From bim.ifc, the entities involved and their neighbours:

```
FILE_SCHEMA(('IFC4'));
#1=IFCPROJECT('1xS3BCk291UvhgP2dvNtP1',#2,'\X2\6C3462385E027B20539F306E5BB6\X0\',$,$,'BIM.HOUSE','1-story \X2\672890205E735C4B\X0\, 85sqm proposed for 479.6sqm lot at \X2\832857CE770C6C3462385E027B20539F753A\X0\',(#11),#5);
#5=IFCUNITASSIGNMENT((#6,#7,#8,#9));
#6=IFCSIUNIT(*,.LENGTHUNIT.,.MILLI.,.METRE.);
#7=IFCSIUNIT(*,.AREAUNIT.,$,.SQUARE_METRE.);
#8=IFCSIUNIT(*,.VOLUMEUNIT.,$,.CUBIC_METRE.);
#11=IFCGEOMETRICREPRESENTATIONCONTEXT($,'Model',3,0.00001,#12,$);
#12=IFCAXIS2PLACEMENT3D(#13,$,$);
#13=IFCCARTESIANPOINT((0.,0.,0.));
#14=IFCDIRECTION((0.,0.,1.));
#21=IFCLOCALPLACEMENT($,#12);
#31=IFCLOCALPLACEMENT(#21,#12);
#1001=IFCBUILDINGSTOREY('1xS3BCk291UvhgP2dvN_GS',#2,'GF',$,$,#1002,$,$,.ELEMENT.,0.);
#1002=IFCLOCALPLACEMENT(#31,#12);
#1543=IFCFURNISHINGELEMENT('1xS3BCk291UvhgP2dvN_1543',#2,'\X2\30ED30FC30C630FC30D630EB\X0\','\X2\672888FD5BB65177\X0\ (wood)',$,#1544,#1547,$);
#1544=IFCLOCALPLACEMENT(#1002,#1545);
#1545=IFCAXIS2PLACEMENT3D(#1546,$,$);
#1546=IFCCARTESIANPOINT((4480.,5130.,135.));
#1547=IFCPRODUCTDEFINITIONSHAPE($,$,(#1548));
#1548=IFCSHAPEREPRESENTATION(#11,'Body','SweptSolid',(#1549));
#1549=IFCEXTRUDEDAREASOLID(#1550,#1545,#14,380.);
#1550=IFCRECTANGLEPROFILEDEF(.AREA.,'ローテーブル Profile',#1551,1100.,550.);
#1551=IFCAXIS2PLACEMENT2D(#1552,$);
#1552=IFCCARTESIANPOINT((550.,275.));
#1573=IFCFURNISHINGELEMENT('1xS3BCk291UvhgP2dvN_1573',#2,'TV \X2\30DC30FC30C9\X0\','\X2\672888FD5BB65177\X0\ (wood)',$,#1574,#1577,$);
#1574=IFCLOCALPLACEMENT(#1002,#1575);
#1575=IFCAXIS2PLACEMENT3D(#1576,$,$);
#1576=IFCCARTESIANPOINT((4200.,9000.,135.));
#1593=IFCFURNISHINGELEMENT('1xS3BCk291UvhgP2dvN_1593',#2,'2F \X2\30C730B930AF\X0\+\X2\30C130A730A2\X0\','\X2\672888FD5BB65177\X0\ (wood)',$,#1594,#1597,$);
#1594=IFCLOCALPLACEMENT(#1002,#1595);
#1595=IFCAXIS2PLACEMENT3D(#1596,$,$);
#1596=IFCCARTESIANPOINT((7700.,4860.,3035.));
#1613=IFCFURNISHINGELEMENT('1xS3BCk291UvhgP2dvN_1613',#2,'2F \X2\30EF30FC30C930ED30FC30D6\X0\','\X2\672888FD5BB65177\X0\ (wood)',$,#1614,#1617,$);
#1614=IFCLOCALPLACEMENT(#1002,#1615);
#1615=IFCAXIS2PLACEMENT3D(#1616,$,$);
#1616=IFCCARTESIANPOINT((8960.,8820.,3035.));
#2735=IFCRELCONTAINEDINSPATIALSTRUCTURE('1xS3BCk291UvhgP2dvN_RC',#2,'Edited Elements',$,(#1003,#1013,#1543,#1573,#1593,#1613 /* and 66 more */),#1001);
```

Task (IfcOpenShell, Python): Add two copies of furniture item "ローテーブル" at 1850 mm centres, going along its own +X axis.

```python
import ifcopenshell
import ifcopenshell.api.geometry
import ifcopenshell.api.root
import ifcopenshell.util.element
import ifcopenshell.util.placement
import ifcopenshell.util.unit

model = ifcopenshell.open("bim.ifc")
unit_scale = ifcopenshell.util.unit.calculate_unit_scale(model)


def reuse_history(source, copy):
    """copy_class also copies each property set's owner history, people and application; keep the originals."""
    for rel in copy.IsDefinedBy:
        if rel.is_a("IfcRelDefinesByProperties") and (history := rel.RelatingPropertyDefinition.OwnerHistory):
            rel.RelatingPropertyDefinition.OwnerHistory = source.OwnerHistory
            ifcopenshell.util.element.remove_deep2(model, history)


source = model.by_guid("1xS3BCk291UvhgP2dvN_1543")
base = ifcopenshell.util.placement.get_local_placement(source.ObjectPlacement)
step = base[:3, 0] * 1.85 / unit_scale

for i in range(1, 3):
    copy = ifcopenshell.api.root.copy_class(model, product=source)
    copy.Representation = ifcopenshell.util.element.copy_deep(
        model, source.Representation, exclude=["IfcGeometricRepresentationContext", "IfcRepresentationMap"]
    )
    reuse_history(source, copy)
    matrix = base.copy()
    matrix[:3, 3] += i * step
    print("added at", matrix[:3, 3].round(3) + 0.0)
    ifcopenshell.api.geometry.edit_object_placement(model, product=copy, matrix=matrix, is_si=False)

model.write("bim_updated.ifc")
```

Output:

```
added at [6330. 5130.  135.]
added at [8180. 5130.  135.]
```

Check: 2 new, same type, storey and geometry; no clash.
